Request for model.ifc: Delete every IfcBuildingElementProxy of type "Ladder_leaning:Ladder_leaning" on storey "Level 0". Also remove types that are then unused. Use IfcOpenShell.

First a look at what the model holds.

```python
import ifcopenshell
import ifcopenshell.util.element

model = ifcopenshell.open("model.ifc")
print(model.schema)
storey = next(s for s in model.by_type("IfcBuildingStorey") if s.Name == "Level 0")
proxies = [e for e in ifcopenshell.util.element.get_decomposition(storey) if e.is_a("IfcBuildingElementProxy")]
seen = {}
for e in proxies:
    element_type = ifcopenshell.util.element.get_type(e)
    name = element_type.Name if element_type not in (None, e) else None
    seen[name] = seen.get(name, 0) + 1
for name, count in sorted(seen.items(), key=str):
    print(count, "x", name)
```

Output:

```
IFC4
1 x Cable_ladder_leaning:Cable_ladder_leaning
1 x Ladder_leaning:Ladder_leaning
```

```python
import ifcopenshell
import ifcopenshell.api.root
import ifcopenshell.util.element

model = ifcopenshell.open("model.ifc")

storey = next(s for s in model.by_type("IfcBuildingStorey") if s.Name == "Level 0")
proxies = [e for e in ifcopenshell.util.element.get_decomposition(storey) if e.is_a("IfcBuildingElementProxy")]
targets = [e for e in proxies if (t := ifcopenshell.util.element.get_type(e)) not in (None, e) and t.Name == "Ladder_leaning:Ladder_leaning"]
types = {ifcopenshell.util.element.get_type(e) for e in targets} - {None, *targets}

for e in targets:
    ifcopenshell.api.root.remove_product(model, product=e)
print(len(targets), "removed")

unused = [t for t in types if not ifcopenshell.util.element.get_types(t)]
for t in unused:
    ifcopenshell.api.root.remove_product(model, product=t)
print(len(unused), "unused types removed")

model.write("model_edited.ifc")
```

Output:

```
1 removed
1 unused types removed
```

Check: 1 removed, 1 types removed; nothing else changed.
